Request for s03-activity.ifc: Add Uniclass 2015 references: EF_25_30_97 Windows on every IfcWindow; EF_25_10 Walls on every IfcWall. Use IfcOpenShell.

First a look at what the model holds.

```python
import ifcopenshell

model = ifcopenshell.open("s03-activity.ifc")
print(model.schema)
print("classifications:", [c.Name for c in model.by_type("IfcClassification")])
for ifc_class in ("IfcDoor", "IfcRoof", "IfcStair", "IfcWall", "IfcWindow"):
    print(ifc_class, len(model.by_type(ifc_class)))
```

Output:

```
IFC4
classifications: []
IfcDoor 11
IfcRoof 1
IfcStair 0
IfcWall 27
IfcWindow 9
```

```python
import ifcopenshell
import ifcopenshell.api.classification

model = ifcopenshell.open("s03-activity.ifc")

system = ifcopenshell.api.classification.add_classification(model, classification="Uniclass 2015")

codes = {
    "IfcWindow": ("EF_25_30_97", "Windows"),
    "IfcWall": ("EF_25_10", "Walls"),
}
for ifc_class, (code, name) in codes.items():
    products = model.by_type(ifc_class)
    ifcopenshell.api.classification.add_reference(
        model, products=products, classification=system, identification=code, name=name
    )
    print(code, len(products))

model.write("s03-activity_v2.ifc")
```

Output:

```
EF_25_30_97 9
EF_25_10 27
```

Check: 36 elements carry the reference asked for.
